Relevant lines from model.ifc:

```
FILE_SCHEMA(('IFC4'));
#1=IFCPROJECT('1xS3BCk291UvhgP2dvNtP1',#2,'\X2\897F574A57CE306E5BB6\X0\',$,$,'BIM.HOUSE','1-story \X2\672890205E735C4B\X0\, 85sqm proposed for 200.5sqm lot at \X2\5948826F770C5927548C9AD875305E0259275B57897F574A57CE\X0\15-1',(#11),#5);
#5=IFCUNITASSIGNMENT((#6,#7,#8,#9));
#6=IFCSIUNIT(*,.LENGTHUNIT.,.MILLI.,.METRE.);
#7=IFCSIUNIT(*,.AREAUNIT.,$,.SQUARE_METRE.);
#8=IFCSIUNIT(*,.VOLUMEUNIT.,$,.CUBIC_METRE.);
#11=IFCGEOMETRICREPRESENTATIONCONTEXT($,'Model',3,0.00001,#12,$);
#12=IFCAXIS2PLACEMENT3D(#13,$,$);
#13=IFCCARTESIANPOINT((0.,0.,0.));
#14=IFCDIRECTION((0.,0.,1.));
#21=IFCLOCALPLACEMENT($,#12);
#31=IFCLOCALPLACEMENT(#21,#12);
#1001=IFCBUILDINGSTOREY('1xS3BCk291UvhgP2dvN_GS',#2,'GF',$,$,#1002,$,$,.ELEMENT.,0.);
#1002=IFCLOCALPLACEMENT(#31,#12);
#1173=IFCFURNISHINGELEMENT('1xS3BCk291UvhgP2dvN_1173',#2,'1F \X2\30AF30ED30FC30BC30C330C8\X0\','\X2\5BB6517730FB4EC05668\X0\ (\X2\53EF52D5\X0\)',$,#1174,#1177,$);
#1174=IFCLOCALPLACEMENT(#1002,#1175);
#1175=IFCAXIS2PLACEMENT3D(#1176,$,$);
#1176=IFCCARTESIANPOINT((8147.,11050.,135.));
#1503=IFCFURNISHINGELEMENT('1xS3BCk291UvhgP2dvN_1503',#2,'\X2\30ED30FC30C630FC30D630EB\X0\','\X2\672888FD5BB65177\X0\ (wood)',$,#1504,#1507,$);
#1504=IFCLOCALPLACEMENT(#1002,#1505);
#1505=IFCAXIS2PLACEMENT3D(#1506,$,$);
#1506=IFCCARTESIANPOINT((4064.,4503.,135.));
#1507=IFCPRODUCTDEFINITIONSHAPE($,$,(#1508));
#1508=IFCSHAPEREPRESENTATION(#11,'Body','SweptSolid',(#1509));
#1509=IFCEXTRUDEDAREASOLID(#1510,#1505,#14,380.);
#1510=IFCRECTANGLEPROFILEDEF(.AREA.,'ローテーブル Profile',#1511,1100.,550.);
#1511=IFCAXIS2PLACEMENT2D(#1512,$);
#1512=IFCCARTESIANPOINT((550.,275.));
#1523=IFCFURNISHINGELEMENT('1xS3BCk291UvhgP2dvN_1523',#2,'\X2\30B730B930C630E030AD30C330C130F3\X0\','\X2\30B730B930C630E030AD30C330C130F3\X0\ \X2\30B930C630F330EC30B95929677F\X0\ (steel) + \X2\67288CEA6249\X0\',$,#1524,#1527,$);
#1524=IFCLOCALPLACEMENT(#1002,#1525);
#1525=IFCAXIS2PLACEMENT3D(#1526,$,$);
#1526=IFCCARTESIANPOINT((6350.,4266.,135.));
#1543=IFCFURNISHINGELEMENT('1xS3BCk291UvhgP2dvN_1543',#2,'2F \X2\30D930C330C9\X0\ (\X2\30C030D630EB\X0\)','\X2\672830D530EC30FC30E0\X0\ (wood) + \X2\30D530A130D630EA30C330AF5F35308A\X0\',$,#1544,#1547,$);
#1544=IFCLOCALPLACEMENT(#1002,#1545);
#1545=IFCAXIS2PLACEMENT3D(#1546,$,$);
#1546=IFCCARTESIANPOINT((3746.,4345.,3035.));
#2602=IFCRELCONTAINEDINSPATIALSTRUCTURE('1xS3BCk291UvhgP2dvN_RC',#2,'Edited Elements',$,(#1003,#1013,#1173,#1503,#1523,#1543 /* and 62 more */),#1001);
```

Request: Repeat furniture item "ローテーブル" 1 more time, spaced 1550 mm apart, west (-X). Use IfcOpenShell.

```python
import numpy as np
import ifcopenshell
import ifcopenshell.api.geometry
import ifcopenshell.api.root
import ifcopenshell.util.element
import ifcopenshell.util.placement
import ifcopenshell.util.unit

model = ifcopenshell.open("model.ifc")
unit_scale = ifcopenshell.util.unit.calculate_unit_scale(model)


def reuse_history(source, copy):
    """copy_class also copies each property set's owner history, people and application; keep the originals."""
    for rel in copy.IsDefinedBy:
        if rel.is_a("IfcRelDefinesByProperties") and (history := rel.RelatingPropertyDefinition.OwnerHistory):
            rel.RelatingPropertyDefinition.OwnerHistory = source.OwnerHistory
            ifcopenshell.util.element.remove_deep2(model, history)


source = model.by_id(1503)
base = ifcopenshell.util.placement.get_local_placement(source.ObjectPlacement)
step = np.array([-1.0, 0.0, 0.0]) * 1.55 / unit_scale

for i in range(1, 2):
    copy = ifcopenshell.api.root.copy_class(model, product=source)
    copy.Representation = ifcopenshell.util.element.copy_deep(
        model, source.Representation, exclude=["IfcGeometricRepresentationContext", "IfcRepresentationMap"]
    )
    reuse_history(source, copy)
    matrix = base.copy()
    matrix[:3, 3] += i * step
    print("added at", matrix[:3, 3].round(3) + 0.0)
    ifcopenshell.api.geometry.edit_object_placement(model, product=copy, matrix=matrix, is_si=False)

model.write("model_rev.ifc")
```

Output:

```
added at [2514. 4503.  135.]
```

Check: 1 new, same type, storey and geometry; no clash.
